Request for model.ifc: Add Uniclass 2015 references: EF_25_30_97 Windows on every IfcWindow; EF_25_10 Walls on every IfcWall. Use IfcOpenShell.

First a look at what the model holds.

```python
import ifcopenshell

model = ifcopenshell.open("model.ifc")
print(model.schema)
print("classifications:", [c.Name for c in model.by_type("IfcClassification")])
for ifc_class in ("IfcDoor", "IfcRoof", "IfcStair", "IfcWall", "IfcWindow"):
    print(ifc_class, len(model.by_type(ifc_class)))
```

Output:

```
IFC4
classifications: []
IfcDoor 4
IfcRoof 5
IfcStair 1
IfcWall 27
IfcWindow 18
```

```python
import ifcopenshell
import ifcopenshell.api.classification

model = ifcopenshell.open("model.ifc")

system = ifcopenshell.api.classification.add_classification(model, classification="Uniclass 2015")

codes = {
    "IfcWindow": ("EF_25_30_97", "Windows"),
    "IfcWall": ("EF_25_10", "Walls"),
}
for ifc_class, (code, name) in codes.items():
    products = model.by_type(ifc_class)
    ifcopenshell.api.classification.add_reference(
        model, products=products, classification=system, identification=code, name=name
    )
    print(code, len(products))

model.write("model_v2.ifc")
```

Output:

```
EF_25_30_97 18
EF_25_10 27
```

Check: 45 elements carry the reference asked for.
